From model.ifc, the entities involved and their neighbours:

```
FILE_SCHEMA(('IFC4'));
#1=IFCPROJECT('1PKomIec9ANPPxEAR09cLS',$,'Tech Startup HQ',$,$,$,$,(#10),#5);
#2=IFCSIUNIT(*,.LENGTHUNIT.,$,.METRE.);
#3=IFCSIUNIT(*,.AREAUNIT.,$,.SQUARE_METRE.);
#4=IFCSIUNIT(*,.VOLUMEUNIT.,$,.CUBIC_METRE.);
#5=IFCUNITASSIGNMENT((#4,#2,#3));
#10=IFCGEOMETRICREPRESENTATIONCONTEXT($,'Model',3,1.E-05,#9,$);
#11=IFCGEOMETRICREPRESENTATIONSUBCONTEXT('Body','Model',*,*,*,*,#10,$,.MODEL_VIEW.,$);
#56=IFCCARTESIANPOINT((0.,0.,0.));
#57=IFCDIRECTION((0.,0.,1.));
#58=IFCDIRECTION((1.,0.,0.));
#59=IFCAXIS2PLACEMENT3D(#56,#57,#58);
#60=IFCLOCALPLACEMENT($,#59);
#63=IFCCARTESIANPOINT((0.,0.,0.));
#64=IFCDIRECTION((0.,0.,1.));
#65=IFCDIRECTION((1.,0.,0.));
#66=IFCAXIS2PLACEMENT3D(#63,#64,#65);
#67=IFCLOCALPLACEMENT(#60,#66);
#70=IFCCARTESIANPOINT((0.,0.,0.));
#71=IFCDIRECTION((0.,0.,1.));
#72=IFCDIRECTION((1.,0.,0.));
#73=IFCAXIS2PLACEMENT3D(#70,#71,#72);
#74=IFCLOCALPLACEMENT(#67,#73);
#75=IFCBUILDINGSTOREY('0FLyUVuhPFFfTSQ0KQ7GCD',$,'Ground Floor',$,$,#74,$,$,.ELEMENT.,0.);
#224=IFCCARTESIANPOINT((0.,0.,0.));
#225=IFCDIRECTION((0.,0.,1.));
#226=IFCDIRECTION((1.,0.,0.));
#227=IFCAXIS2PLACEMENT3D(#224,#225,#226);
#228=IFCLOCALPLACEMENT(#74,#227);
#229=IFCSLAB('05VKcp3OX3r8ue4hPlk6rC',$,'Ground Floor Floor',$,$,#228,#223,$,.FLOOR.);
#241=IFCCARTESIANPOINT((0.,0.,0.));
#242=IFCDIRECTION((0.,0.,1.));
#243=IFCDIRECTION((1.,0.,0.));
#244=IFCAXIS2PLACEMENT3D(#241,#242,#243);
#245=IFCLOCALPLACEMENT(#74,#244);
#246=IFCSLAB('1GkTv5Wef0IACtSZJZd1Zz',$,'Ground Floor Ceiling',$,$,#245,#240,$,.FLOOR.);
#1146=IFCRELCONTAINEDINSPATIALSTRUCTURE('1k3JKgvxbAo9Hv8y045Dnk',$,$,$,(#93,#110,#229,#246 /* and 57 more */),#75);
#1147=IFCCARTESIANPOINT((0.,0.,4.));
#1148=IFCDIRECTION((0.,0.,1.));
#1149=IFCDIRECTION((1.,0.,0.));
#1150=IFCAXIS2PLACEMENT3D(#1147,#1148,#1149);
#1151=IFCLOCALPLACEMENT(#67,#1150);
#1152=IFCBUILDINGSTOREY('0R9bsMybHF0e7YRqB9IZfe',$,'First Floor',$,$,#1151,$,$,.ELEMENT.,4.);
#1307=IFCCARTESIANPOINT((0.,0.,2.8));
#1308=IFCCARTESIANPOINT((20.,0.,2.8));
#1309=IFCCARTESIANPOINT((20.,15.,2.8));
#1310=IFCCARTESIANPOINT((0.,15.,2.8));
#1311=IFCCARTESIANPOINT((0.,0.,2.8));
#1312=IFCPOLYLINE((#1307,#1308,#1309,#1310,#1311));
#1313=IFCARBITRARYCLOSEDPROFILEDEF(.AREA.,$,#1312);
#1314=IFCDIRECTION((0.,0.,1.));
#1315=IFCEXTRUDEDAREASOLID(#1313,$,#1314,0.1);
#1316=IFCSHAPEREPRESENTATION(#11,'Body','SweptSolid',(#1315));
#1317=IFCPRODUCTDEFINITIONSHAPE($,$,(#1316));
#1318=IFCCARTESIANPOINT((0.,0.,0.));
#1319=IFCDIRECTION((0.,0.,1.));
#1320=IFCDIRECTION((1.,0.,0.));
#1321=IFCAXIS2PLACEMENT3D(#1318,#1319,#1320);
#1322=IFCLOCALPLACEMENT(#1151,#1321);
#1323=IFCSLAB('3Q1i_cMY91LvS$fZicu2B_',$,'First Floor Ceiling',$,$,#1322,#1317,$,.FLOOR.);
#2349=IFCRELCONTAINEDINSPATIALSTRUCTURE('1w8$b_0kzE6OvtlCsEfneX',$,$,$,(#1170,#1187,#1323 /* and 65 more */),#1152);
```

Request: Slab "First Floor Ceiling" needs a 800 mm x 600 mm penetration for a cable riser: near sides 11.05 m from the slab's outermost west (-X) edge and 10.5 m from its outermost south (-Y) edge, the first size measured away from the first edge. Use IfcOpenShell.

```python
import numpy as np
import ifcopenshell
import ifcopenshell.api.feature
import ifcopenshell.api.geometry
import ifcopenshell.api.root
import ifcopenshell.geom
import ifcopenshell.util.placement
import ifcopenshell.util.representation
import ifcopenshell.util.shape
import ifcopenshell.util.unit

model = ifcopenshell.open("model.ifc")
unit_scale = ifcopenshell.util.unit.calculate_unit_scale(model)
settings = ifcopenshell.geom.settings()


def volume(element):
    """Net volume in cubic metres, openings subtracted."""
    shape = ifcopenshell.geom.create_shape(settings, element)
    return ifcopenshell.util.shape.get_volume(shape.geometry)


slab = model.by_guid("3Q1i_cMY91LvS$fZicu2B_")
before = volume(slab)

# Extent in the slab's own axes, in metres. The edges named are its -X and -Y sides.
slab_shape = ifcopenshell.geom.create_shape(settings, slab)
vertices = ifcopenshell.util.shape.get_vertices(slab_shape.geometry)
x_min, y_min, bottom = vertices.min(axis=0)
top = vertices[:, 2].max()

opening = ifcopenshell.api.root.create_entity(model, ifc_class="IfcOpeningElement", name="Cable riser opening", predefined_type="OPENING")
context = ifcopenshell.util.representation.get_context(model, "Model", "Body", "MODEL_VIEW")
width, depth = 0.8, 0.6
outline = [(0.0, 0.0), (width, 0.0), (width, depth), (0.0, depth), (0.0, 0.0)]
# Overshoot both faces by 50 mm so the cut is clean.
shape = ifcopenshell.api.geometry.add_slab_representation(
    model, context=context, depth=top - bottom + 0.1, polyline=outline
)
ifcopenshell.api.geometry.assign_representation(model, product=opening, representation=shape)

matrix = ifcopenshell.util.placement.get_local_placement(slab.ObjectPlacement)
matrix[:, 3] = matrix @ np.append(np.array([x_min + 11.05, y_min + 10.5, bottom - 0.05]) / unit_scale, 1.0)
ifcopenshell.api.geometry.edit_object_placement(model, product=opening, matrix=matrix, is_si=False)
ifcopenshell.api.feature.add_feature(model, feature=opening, element=slab)

after = volume(slab)

print(f"slab volume {before:.3f} -> {after:.3f} m3")

model.write("model-out.ifc")
```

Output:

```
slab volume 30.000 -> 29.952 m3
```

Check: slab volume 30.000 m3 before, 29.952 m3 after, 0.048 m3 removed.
